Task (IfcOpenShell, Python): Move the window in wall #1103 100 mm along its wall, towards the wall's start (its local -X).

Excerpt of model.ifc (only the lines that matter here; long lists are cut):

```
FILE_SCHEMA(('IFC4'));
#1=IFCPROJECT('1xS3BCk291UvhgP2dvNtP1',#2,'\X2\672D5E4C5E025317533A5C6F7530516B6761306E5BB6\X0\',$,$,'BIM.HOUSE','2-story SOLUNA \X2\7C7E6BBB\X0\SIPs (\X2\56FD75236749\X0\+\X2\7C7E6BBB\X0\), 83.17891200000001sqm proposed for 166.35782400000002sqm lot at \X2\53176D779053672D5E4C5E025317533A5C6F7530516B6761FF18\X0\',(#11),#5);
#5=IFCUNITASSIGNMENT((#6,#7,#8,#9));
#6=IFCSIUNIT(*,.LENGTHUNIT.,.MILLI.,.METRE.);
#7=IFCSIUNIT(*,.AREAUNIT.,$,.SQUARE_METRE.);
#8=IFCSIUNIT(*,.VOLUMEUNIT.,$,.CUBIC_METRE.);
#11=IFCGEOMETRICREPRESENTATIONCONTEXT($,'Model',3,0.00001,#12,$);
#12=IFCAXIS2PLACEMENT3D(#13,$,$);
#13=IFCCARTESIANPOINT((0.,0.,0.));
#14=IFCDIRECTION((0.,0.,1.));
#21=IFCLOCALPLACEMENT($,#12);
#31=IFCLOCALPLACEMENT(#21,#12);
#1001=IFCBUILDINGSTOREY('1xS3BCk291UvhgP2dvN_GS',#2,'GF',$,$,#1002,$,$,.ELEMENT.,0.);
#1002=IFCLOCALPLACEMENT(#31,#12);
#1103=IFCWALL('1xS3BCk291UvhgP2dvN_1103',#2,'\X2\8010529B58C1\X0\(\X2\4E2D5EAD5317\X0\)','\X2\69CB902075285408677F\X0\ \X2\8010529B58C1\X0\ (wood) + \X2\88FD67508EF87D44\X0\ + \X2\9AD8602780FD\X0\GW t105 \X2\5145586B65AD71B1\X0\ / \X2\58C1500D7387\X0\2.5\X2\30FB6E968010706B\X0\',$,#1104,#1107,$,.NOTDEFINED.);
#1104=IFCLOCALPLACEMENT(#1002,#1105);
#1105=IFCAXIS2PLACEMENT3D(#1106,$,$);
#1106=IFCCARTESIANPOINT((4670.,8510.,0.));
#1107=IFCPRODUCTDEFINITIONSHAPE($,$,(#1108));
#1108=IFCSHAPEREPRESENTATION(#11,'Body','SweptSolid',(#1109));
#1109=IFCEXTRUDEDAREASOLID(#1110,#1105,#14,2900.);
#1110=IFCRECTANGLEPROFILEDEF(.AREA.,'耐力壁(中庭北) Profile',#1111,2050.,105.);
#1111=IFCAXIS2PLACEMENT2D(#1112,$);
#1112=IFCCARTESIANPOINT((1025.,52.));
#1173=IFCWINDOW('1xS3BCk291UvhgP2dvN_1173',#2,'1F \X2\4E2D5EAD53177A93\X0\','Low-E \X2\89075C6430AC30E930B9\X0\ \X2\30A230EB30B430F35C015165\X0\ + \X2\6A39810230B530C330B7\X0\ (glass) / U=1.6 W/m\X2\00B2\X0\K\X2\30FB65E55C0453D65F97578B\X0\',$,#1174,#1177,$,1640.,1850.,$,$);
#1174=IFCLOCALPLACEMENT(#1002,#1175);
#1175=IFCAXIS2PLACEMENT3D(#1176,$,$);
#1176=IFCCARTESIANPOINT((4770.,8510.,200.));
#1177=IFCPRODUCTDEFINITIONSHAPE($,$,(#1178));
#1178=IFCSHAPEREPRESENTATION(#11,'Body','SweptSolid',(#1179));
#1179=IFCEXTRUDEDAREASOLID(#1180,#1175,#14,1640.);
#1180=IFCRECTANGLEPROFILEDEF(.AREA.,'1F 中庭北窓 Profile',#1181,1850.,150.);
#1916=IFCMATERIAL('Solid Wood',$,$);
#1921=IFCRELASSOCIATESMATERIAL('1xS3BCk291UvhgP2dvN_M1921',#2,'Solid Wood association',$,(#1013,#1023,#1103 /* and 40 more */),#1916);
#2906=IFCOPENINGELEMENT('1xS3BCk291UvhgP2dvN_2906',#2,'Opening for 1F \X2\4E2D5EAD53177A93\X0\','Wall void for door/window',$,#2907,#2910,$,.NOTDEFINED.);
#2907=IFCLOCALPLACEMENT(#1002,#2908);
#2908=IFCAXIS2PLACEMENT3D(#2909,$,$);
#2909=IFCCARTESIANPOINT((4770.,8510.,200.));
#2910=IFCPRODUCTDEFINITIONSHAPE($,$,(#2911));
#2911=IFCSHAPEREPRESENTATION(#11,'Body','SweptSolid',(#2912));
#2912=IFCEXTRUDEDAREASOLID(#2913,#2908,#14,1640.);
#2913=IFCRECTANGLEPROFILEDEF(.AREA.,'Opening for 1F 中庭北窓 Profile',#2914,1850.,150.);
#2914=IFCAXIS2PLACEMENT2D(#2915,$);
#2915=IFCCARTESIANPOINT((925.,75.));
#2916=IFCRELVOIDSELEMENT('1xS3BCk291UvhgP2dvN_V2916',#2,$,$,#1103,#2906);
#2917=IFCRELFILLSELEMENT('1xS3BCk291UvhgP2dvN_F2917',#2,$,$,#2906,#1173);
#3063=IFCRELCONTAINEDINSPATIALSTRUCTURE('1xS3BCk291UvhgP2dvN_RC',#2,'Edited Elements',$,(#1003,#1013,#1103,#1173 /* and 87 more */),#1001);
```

```python
import ifcopenshell
import ifcopenshell.api.geometry
import ifcopenshell.util.placement

model = ifcopenshell.open("model.ifc")

window = model.by_guid("1xS3BCk291UvhgP2dvN_1173")
opening = window.FillsVoids[0].RelatingOpeningElement
wall = opening.VoidsElements[0].RelatingBuildingElement

wall_matrix = ifcopenshell.util.placement.get_local_placement(wall.ObjectPlacement)
shift = wall_matrix[:3, 0] * -100.0
before = ifcopenshell.util.placement.get_local_placement(window.ObjectPlacement)[:3, 3].copy()

# The window is not placed relative to its opening, so move both.
for product in (opening, window):
    matrix = ifcopenshell.util.placement.get_local_placement(product.ObjectPlacement)
    matrix[:3, 3] += shift
    ifcopenshell.api.geometry.edit_object_placement(model, product=product, matrix=matrix, is_si=False)

after = ifcopenshell.util.placement.get_local_placement(window.ObjectPlacement)[:3, 3]
print("window moved by", (after - before).round(3) + 0.0)

model.write("model_v2.ifc")
```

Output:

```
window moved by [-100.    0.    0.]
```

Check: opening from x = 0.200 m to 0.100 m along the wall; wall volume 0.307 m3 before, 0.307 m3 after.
